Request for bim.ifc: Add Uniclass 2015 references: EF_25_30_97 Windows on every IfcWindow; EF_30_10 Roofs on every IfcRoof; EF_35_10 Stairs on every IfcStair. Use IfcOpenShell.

First a look at what the model holds.

```python
import ifcopenshell

model = ifcopenshell.open("bim.ifc")
print(model.schema)
print("classifications:", [c.Name for c in model.by_type("IfcClassification")])
for ifc_class in ("IfcDoor", "IfcRoof", "IfcStair", "IfcWall", "IfcWindow"):
    print(ifc_class, len(model.by_type(ifc_class)))
```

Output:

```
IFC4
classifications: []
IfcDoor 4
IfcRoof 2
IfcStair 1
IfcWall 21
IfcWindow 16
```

```python
import ifcopenshell
import ifcopenshell.api.classification

model = ifcopenshell.open("bim.ifc")

system = ifcopenshell.api.classification.add_classification(model, classification="Uniclass 2015")

codes = {
    "IfcWindow": ("EF_25_30_97", "Windows"),
    "IfcRoof": ("EF_30_10", "Roofs"),
    "IfcStair": ("EF_35_10", "Stairs"),
}
for ifc_class, (code, name) in codes.items():
    products = model.by_type(ifc_class)
    ifcopenshell.api.classification.add_reference(
        model, products=products, classification=system, identification=code, name=name
    )
    print(code, len(products))

model.write("bim_updated.ifc")
```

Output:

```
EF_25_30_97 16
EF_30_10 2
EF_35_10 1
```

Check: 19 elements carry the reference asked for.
